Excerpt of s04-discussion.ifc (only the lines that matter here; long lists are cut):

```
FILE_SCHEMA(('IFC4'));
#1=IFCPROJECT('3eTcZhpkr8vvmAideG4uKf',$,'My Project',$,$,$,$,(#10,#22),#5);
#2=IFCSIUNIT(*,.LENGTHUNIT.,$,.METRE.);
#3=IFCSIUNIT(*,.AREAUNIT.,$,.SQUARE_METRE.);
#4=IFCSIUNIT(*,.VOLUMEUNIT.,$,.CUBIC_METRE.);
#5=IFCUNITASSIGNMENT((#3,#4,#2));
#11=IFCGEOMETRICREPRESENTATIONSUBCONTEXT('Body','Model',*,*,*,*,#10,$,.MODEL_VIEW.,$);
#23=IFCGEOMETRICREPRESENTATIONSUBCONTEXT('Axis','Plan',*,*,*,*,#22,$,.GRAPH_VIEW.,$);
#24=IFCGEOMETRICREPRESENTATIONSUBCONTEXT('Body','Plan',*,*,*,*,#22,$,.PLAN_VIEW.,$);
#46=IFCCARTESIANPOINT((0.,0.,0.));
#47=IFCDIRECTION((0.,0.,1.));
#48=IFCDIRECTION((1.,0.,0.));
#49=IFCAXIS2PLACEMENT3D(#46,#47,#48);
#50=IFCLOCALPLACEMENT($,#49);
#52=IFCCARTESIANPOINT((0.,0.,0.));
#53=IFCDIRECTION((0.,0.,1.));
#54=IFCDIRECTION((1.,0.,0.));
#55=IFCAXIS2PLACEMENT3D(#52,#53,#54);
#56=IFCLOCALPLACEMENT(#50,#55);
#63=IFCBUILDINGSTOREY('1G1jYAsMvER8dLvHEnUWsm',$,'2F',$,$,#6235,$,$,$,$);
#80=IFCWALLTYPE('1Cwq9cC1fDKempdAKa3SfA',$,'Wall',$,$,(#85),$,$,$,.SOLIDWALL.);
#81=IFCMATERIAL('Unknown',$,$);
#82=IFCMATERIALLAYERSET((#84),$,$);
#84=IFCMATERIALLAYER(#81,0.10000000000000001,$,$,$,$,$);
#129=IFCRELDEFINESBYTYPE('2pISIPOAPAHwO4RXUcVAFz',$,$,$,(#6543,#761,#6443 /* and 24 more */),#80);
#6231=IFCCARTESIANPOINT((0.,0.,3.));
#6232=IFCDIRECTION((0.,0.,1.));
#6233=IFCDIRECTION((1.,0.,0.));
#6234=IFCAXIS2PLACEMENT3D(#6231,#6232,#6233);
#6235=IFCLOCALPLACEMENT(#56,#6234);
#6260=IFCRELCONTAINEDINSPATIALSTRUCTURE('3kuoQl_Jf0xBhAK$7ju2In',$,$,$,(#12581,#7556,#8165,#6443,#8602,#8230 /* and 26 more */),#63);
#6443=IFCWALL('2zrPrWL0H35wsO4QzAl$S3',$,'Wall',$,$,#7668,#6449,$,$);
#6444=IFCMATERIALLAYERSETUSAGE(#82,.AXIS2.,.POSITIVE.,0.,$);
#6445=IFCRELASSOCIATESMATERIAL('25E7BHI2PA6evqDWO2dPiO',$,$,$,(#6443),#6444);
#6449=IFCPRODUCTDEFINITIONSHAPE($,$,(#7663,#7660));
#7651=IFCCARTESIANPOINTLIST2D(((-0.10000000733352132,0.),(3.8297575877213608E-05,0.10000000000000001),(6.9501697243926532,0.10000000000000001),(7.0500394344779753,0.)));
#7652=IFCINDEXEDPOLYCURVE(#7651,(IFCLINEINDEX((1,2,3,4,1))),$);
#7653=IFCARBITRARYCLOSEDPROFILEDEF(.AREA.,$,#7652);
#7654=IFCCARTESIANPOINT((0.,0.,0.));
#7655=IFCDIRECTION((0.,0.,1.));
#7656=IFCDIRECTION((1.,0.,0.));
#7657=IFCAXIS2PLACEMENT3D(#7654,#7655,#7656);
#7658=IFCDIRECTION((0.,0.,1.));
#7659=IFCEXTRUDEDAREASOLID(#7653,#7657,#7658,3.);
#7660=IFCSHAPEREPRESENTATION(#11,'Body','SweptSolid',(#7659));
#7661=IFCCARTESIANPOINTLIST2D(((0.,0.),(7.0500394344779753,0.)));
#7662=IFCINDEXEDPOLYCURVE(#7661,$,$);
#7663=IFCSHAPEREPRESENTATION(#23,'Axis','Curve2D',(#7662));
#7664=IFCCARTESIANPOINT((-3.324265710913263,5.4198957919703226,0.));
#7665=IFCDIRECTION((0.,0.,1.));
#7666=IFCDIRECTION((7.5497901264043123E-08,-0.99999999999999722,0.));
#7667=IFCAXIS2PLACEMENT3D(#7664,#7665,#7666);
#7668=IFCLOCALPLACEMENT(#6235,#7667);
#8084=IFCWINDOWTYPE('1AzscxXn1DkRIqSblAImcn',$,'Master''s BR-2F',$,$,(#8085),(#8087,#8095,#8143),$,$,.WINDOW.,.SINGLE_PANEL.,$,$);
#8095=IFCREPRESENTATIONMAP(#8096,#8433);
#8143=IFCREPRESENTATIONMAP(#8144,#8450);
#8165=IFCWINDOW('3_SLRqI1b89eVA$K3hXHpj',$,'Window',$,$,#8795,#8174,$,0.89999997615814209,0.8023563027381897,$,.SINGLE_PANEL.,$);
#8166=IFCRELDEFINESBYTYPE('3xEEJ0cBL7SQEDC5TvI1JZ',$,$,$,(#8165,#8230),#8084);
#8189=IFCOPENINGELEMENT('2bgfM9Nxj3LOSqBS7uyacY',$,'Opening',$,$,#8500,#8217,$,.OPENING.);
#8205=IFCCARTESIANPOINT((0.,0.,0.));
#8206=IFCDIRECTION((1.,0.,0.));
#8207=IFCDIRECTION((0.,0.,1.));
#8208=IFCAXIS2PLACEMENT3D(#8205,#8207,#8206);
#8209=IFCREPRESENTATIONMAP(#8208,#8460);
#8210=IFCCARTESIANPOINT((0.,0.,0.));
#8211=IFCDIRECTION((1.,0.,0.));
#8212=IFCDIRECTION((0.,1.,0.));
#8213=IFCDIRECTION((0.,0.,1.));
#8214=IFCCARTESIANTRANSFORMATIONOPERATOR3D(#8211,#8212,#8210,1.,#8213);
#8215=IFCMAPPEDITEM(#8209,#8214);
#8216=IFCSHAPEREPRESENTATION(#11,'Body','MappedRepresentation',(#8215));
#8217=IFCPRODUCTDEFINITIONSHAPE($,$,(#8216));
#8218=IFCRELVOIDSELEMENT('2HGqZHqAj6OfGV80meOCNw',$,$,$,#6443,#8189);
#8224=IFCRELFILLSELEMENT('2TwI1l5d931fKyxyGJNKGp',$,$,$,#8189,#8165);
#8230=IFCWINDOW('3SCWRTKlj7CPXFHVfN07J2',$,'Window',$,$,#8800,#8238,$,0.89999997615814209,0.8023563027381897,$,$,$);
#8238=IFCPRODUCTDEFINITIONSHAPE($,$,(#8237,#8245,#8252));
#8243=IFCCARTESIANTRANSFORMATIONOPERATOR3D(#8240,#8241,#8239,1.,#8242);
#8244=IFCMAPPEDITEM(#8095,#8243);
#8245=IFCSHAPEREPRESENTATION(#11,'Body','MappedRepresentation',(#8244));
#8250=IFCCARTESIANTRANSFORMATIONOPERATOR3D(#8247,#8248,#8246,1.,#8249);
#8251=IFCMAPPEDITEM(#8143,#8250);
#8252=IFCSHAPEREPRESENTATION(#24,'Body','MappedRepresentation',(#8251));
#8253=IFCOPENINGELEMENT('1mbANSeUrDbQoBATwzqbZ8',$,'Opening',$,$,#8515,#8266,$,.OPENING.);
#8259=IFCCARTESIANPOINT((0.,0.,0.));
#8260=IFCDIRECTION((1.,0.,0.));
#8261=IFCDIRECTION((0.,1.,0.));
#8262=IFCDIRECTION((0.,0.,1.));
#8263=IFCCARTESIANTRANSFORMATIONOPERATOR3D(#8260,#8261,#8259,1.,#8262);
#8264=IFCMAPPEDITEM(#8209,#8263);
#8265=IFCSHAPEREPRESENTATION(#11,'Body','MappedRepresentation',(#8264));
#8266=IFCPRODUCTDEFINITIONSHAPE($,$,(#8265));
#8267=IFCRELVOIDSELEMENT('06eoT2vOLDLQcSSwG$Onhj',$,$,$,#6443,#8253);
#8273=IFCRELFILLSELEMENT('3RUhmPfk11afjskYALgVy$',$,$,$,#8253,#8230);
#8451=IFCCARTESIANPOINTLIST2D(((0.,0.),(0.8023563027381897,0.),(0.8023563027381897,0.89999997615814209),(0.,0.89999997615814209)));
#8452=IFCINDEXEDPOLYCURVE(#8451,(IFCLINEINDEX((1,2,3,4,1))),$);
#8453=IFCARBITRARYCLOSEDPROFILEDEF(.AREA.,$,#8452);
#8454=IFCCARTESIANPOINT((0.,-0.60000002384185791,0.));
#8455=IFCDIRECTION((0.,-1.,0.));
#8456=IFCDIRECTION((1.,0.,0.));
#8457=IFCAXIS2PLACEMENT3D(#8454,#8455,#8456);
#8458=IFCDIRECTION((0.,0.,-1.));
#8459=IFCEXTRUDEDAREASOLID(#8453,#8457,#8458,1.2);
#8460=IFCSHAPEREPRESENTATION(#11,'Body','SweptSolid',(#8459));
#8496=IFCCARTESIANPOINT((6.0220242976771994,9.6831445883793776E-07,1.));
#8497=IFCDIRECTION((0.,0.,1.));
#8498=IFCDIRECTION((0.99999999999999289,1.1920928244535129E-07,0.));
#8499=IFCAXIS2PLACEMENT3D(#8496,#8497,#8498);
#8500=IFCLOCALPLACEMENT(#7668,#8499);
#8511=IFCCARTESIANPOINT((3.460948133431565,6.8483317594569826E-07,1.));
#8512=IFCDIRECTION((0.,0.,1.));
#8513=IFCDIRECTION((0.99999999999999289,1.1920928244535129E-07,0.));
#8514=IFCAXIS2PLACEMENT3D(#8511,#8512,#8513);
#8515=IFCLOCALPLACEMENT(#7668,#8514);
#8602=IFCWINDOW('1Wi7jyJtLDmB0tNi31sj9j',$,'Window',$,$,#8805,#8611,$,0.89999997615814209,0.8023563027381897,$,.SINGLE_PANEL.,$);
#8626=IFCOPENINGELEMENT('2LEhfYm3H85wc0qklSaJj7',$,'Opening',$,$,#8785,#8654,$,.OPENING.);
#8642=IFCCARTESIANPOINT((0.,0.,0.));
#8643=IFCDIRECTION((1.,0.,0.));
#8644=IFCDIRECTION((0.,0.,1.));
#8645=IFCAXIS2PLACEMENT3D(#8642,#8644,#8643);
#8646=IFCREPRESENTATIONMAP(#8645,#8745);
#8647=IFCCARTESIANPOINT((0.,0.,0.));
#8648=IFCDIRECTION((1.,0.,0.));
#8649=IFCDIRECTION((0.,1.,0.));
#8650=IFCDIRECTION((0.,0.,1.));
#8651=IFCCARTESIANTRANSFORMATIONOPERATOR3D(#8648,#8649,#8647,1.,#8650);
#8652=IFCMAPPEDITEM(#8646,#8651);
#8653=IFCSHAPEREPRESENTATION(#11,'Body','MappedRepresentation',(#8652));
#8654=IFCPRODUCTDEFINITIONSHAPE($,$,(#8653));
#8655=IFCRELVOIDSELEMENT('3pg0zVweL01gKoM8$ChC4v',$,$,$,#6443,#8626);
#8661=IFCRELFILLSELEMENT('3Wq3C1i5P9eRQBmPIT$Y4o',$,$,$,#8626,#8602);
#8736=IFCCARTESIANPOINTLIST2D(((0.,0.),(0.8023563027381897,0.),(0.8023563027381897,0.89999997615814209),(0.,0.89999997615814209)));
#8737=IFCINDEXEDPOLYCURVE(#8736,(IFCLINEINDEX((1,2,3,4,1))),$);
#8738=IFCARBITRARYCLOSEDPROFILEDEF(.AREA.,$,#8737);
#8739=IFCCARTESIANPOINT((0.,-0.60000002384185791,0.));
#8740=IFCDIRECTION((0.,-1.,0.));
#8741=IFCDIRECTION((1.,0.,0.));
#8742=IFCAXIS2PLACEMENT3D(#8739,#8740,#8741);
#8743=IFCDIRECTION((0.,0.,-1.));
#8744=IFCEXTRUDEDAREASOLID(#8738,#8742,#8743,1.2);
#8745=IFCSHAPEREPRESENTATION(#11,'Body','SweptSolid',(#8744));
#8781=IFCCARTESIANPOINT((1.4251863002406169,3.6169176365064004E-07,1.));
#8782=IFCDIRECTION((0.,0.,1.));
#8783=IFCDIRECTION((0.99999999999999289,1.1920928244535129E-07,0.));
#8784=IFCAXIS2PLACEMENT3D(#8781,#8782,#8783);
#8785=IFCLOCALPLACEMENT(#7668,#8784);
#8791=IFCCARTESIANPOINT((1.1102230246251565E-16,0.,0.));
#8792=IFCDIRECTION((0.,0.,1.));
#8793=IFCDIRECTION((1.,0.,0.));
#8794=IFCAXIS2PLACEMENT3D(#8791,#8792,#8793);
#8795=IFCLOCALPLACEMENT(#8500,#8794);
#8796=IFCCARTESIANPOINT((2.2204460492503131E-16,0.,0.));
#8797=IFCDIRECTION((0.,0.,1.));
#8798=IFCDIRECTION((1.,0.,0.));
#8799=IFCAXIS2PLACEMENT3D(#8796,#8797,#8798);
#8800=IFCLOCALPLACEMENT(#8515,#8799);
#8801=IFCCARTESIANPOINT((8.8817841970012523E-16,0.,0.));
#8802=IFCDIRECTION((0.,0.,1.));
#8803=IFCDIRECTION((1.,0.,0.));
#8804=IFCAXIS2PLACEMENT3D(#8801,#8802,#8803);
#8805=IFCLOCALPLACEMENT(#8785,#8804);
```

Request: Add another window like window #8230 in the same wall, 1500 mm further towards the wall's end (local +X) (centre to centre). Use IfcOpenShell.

```python
import ifcopenshell
import ifcopenshell.api.feature
import ifcopenshell.api.geometry
import ifcopenshell.api.root
import ifcopenshell.geom
import ifcopenshell.util.element
import ifcopenshell.util.placement
import ifcopenshell.util.shape

model = ifcopenshell.open("s04-discussion.ifc")
settings = ifcopenshell.geom.settings()


def volume(element):
    """Net volume in cubic metres, openings subtracted."""
    shape = ifcopenshell.geom.create_shape(settings, element)
    return ifcopenshell.util.shape.get_volume(shape.geometry)


window = model.by_guid("3SCWRTKlj7CPXFHVfN07J2")
opening = window.FillsVoids[0].RelatingOpeningElement
wall = opening.VoidsElements[0].RelatingBuildingElement
before = volume(wall)
shift = ifcopenshell.util.placement.get_local_placement(wall.ObjectPlacement)[:3, 0] * 1.5

# copy_class copies the void relationship, type, container and properties, but no geometry.
new_opening = ifcopenshell.api.root.copy_class(model, product=opening)
new_opening.Representation = ifcopenshell.util.element.copy_deep(
    model, opening.Representation, exclude=["IfcGeometricRepresentationContext", "IfcRepresentationMap"]
)
new_window = ifcopenshell.api.root.copy_class(model, product=window)
new_window.Representation = ifcopenshell.util.element.copy_deep(
    model, window.Representation, exclude=["IfcGeometricRepresentationContext", "IfcRepresentationMap"]
)
ifcopenshell.api.feature.add_filling(model, opening=new_opening, element=new_window)

for old, new in ((opening, new_opening), (window, new_window)):
    matrix = ifcopenshell.util.placement.get_local_placement(old.ObjectPlacement)
    matrix[:3, 3] += shift
    ifcopenshell.api.geometry.edit_object_placement(model, product=new, matrix=matrix, is_si=False)

after = volume(wall)

print(f"wall volume {before:.3f} -> {after:.3f} m3")

model.write("s04-discussion_v2.ifc")
```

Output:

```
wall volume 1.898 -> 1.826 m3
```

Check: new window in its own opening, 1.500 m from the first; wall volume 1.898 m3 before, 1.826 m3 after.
